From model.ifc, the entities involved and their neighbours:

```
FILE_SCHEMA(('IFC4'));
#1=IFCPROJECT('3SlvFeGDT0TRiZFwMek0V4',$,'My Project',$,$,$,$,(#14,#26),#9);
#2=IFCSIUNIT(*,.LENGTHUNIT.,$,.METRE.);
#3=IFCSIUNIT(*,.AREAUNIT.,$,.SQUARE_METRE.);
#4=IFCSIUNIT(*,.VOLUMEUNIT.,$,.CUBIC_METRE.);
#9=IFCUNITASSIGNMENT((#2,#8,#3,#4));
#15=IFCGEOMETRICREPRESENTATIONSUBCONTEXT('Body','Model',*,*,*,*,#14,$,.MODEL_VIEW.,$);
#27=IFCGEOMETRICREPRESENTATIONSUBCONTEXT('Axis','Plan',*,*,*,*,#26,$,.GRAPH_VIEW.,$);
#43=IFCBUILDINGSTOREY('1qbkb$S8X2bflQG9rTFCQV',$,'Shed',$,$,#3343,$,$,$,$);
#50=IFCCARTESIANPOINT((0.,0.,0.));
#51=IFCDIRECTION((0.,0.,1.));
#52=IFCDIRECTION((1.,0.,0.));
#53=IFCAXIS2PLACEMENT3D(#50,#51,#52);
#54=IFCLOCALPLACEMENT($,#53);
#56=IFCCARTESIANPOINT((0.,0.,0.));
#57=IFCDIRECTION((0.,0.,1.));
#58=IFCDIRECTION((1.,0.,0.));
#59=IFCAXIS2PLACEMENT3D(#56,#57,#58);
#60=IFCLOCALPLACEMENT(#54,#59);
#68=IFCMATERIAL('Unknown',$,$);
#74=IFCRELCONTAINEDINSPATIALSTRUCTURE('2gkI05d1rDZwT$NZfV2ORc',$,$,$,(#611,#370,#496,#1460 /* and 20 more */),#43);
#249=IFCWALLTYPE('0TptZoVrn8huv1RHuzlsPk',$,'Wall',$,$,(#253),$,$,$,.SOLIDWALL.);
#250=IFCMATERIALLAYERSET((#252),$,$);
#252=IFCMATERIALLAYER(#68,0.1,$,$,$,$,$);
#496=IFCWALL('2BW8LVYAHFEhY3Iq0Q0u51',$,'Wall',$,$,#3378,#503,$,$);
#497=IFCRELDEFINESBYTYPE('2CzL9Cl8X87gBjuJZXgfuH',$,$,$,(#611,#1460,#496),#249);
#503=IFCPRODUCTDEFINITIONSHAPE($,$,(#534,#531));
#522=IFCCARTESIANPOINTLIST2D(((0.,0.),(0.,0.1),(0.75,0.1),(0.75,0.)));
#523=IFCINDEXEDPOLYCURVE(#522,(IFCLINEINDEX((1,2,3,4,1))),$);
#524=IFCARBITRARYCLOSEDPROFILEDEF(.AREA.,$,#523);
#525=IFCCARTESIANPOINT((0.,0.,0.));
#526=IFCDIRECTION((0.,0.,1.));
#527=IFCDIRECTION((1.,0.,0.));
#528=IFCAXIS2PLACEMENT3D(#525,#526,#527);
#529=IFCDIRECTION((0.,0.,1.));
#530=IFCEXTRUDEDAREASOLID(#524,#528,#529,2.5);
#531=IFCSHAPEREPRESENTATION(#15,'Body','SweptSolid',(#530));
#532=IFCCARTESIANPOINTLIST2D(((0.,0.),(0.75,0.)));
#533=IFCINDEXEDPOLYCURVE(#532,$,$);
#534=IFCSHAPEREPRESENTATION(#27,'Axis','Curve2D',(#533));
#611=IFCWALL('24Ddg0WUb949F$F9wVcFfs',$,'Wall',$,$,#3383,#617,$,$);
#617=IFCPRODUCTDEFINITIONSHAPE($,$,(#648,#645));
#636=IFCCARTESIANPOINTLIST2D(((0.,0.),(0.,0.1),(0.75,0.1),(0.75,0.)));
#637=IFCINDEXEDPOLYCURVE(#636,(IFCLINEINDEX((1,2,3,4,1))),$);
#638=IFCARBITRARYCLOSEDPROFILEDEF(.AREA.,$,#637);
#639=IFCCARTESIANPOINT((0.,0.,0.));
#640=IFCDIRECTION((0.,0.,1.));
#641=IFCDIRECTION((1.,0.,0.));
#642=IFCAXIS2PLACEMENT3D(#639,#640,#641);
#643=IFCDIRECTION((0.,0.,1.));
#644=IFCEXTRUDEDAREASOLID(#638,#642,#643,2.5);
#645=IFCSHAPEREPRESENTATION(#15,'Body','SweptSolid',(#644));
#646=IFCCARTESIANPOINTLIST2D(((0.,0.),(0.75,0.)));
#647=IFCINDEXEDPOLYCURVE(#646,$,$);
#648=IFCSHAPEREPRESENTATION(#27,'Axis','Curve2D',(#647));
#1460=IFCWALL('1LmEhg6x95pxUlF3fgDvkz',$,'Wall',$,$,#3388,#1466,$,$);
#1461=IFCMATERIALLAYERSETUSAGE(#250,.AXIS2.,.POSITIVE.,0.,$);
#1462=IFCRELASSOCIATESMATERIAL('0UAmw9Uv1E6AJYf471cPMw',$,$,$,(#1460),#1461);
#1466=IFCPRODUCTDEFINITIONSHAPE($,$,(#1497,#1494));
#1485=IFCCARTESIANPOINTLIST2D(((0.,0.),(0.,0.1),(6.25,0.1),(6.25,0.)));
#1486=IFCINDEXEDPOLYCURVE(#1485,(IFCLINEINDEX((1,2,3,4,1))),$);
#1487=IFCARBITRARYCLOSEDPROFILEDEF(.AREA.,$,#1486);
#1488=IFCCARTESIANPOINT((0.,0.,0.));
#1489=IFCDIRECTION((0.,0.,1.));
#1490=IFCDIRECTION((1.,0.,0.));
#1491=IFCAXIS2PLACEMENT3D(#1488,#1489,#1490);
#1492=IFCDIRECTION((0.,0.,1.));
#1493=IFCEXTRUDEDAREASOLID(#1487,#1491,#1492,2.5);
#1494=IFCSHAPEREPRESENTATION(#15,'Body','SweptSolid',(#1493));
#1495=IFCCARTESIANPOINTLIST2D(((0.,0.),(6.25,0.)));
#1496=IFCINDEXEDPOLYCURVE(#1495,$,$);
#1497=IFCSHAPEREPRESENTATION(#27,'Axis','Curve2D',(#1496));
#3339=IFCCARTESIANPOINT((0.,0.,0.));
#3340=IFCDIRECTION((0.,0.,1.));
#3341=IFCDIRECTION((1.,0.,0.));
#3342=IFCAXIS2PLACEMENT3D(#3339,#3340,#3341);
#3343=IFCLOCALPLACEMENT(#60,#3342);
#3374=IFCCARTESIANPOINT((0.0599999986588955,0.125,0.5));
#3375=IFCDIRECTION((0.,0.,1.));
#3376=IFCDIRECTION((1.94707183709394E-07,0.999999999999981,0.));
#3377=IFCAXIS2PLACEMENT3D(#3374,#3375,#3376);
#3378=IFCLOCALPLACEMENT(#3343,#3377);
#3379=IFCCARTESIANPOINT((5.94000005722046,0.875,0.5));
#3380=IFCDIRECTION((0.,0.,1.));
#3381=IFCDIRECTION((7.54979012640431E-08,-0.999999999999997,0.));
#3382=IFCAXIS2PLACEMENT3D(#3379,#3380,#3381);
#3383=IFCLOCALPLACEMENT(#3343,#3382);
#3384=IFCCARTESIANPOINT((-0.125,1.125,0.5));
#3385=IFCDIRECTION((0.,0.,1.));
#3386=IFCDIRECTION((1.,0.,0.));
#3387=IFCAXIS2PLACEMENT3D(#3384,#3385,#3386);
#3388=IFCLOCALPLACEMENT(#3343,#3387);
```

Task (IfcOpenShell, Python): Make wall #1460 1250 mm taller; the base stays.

```python
import ifcopenshell
import ifcopenshell.geom
import ifcopenshell.util.representation
import ifcopenshell.util.shape
import ifcopenshell.util.unit

model = ifcopenshell.open("model.ifc")
unit_scale = ifcopenshell.util.unit.calculate_unit_scale(model)
settings = ifcopenshell.geom.settings()


def volume(element):
    """Net volume in cubic metres, openings subtracted."""
    shape = ifcopenshell.geom.create_shape(settings, element)
    return ifcopenshell.util.shape.get_volume(shape.geometry)


wall = model.by_guid("1LmEhg6x95pxUlF3fgDvkz")
before = volume(wall)

body = ifcopenshell.util.representation.get_representation(wall, "Model", "Body")
solid = body.Items[0]
old_height = solid.Depth
solid.Depth += 1.25 / unit_scale
after = volume(wall)

print(f"height {old_height:g} -> {solid.Depth:g}, volume {before:.3f} -> {after:.3f} m3")

model.write("model_v2.ifc")
```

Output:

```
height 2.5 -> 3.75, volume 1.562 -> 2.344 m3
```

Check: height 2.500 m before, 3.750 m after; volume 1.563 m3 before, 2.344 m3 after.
